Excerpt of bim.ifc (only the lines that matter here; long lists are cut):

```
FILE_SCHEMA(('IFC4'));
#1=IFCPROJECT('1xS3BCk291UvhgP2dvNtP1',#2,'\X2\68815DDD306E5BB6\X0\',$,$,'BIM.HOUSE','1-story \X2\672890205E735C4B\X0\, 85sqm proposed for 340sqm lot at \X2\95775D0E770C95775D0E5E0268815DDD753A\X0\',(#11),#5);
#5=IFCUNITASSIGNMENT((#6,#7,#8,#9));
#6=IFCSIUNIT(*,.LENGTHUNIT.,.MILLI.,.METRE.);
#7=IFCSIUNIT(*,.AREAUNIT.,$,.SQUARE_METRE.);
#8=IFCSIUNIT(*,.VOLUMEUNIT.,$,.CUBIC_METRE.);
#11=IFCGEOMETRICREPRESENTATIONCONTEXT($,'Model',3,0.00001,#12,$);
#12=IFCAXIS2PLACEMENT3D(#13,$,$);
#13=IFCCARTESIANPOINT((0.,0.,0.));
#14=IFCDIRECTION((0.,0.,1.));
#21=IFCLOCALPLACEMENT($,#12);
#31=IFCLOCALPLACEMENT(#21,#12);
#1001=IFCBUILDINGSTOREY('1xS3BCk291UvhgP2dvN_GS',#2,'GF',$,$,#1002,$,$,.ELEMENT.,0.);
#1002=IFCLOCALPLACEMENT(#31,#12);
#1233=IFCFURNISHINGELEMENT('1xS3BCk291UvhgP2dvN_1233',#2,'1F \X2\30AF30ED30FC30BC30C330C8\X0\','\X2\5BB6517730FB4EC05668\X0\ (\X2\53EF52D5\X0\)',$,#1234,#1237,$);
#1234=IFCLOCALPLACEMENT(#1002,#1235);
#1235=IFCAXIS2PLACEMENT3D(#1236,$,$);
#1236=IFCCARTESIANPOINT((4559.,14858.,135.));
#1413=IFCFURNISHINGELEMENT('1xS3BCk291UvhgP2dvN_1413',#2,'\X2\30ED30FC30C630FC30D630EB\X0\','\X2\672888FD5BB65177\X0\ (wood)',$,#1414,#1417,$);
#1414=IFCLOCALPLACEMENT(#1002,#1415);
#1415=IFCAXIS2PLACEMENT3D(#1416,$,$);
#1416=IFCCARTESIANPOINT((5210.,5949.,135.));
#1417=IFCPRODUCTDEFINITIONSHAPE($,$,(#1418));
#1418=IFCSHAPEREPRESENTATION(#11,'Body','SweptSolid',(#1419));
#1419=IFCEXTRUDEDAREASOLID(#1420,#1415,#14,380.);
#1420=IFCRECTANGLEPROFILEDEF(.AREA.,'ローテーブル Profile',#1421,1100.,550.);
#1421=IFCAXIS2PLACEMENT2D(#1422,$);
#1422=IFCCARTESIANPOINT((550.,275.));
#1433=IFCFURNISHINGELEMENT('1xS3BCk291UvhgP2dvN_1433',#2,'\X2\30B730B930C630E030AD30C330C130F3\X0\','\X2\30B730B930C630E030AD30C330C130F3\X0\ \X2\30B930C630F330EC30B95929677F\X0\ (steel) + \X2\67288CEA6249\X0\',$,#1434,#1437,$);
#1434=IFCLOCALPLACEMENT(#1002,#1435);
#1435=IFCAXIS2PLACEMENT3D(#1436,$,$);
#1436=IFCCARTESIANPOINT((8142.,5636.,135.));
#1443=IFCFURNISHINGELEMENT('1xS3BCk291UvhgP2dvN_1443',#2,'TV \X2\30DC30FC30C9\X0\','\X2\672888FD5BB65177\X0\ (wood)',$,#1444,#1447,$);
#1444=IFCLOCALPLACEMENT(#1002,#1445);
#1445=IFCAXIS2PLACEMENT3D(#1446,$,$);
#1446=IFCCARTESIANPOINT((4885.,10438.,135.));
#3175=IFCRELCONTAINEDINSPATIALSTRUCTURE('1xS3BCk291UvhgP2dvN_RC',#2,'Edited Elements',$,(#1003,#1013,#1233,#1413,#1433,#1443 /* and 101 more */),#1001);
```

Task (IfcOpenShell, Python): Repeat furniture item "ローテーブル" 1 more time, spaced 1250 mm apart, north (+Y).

```python
import numpy as np
import ifcopenshell
import ifcopenshell.api.geometry
import ifcopenshell.api.root
import ifcopenshell.util.element
import ifcopenshell.util.placement
import ifcopenshell.util.unit

model = ifcopenshell.open("bim.ifc")
unit_scale = ifcopenshell.util.unit.calculate_unit_scale(model)


def reuse_history(source, copy):
    """copy_class also copies each property set's owner history, people and application; keep the originals."""
    for rel in copy.IsDefinedBy:
        if rel.is_a("IfcRelDefinesByProperties") and (history := rel.RelatingPropertyDefinition.OwnerHistory):
            rel.RelatingPropertyDefinition.OwnerHistory = source.OwnerHistory
            ifcopenshell.util.element.remove_deep2(model, history)


source = model.by_guid("1xS3BCk291UvhgP2dvN_1413")
base = ifcopenshell.util.placement.get_local_placement(source.ObjectPlacement)
step = np.array([0.0, 1.0, 0.0]) * 1.25 / unit_scale

for i in range(1, 2):
    copy = ifcopenshell.api.root.copy_class(model, product=source)
    copy.Representation = ifcopenshell.util.element.copy_deep(
        model, source.Representation, exclude=["IfcGeometricRepresentationContext", "IfcRepresentationMap"]
    )
    reuse_history(source, copy)
    matrix = base.copy()
    matrix[:3, 3] += i * step
    print("added at", matrix[:3, 3].round(3) + 0.0)
    ifcopenshell.api.geometry.edit_object_placement(model, product=copy, matrix=matrix, is_si=False)

model.write("bim_rev.ifc")
```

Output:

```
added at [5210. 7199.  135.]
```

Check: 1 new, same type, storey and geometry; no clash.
